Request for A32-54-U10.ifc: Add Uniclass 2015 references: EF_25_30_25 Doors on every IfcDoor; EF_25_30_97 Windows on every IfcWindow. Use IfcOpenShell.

First a look at what the model holds.

```python
import ifcopenshell

model = ifcopenshell.open("A32-54-U10.ifc")
print(model.schema)
print("classifications:", [c.Name for c in model.by_type("IfcClassification")])
for ifc_class in ("IfcDoor", "IfcRoof", "IfcStair", "IfcWall", "IfcWindow"):
    print(ifc_class, len(model.by_type(ifc_class)))
```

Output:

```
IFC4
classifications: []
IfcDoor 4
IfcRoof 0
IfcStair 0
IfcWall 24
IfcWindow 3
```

```python
import ifcopenshell
import ifcopenshell.api.classification

model = ifcopenshell.open("A32-54-U10.ifc")

system = ifcopenshell.api.classification.add_classification(model, classification="Uniclass 2015")

codes = {
    "IfcDoor": ("EF_25_30_25", "Doors"),
    "IfcWindow": ("EF_25_30_97", "Windows"),
}
for ifc_class, (code, name) in codes.items():
    products = model.by_type(ifc_class)
    ifcopenshell.api.classification.add_reference(
        model, products=products, classification=system, identification=code, name=name
    )
    print(code, len(products))

model.write("A32-54-U10_v2.ifc")
```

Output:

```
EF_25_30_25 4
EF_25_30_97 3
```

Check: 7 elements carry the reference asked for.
